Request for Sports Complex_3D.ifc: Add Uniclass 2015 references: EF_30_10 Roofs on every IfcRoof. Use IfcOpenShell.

First a look at what the model holds.

```python
import ifcopenshell

model = ifcopenshell.open("Sports Complex_3D.ifc")
print(model.schema)
print("classifications:", [c.Name for c in model.by_type("IfcClassification")])
for ifc_class in ("IfcDoor", "IfcRoof", "IfcStair", "IfcWall", "IfcWindow"):
    print(ifc_class, len(model.by_type(ifc_class)))
```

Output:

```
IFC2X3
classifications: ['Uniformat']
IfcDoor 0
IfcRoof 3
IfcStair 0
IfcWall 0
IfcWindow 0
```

```python
import ifcopenshell
import ifcopenshell.api.classification

model = ifcopenshell.open("Sports Complex_3D.ifc")

# IFC2X3 requires Source and Edition and has no link from the project to the system.
system = model.create_entity("IfcClassification", Source="NBS", Edition="2015", Name="Uniclass 2015")

codes = {
    "IfcRoof": ("EF_30_10", "Roofs"),
}
for ifc_class, (code, name) in codes.items():
    products = model.by_type(ifc_class)
    ifcopenshell.api.classification.add_reference(
        model, products=products, classification=system, identification=code, name=name
    )
    print(code, len(products))

model.write("Sports Complex_3D_edited.ifc")
```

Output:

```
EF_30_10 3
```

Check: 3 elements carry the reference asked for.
